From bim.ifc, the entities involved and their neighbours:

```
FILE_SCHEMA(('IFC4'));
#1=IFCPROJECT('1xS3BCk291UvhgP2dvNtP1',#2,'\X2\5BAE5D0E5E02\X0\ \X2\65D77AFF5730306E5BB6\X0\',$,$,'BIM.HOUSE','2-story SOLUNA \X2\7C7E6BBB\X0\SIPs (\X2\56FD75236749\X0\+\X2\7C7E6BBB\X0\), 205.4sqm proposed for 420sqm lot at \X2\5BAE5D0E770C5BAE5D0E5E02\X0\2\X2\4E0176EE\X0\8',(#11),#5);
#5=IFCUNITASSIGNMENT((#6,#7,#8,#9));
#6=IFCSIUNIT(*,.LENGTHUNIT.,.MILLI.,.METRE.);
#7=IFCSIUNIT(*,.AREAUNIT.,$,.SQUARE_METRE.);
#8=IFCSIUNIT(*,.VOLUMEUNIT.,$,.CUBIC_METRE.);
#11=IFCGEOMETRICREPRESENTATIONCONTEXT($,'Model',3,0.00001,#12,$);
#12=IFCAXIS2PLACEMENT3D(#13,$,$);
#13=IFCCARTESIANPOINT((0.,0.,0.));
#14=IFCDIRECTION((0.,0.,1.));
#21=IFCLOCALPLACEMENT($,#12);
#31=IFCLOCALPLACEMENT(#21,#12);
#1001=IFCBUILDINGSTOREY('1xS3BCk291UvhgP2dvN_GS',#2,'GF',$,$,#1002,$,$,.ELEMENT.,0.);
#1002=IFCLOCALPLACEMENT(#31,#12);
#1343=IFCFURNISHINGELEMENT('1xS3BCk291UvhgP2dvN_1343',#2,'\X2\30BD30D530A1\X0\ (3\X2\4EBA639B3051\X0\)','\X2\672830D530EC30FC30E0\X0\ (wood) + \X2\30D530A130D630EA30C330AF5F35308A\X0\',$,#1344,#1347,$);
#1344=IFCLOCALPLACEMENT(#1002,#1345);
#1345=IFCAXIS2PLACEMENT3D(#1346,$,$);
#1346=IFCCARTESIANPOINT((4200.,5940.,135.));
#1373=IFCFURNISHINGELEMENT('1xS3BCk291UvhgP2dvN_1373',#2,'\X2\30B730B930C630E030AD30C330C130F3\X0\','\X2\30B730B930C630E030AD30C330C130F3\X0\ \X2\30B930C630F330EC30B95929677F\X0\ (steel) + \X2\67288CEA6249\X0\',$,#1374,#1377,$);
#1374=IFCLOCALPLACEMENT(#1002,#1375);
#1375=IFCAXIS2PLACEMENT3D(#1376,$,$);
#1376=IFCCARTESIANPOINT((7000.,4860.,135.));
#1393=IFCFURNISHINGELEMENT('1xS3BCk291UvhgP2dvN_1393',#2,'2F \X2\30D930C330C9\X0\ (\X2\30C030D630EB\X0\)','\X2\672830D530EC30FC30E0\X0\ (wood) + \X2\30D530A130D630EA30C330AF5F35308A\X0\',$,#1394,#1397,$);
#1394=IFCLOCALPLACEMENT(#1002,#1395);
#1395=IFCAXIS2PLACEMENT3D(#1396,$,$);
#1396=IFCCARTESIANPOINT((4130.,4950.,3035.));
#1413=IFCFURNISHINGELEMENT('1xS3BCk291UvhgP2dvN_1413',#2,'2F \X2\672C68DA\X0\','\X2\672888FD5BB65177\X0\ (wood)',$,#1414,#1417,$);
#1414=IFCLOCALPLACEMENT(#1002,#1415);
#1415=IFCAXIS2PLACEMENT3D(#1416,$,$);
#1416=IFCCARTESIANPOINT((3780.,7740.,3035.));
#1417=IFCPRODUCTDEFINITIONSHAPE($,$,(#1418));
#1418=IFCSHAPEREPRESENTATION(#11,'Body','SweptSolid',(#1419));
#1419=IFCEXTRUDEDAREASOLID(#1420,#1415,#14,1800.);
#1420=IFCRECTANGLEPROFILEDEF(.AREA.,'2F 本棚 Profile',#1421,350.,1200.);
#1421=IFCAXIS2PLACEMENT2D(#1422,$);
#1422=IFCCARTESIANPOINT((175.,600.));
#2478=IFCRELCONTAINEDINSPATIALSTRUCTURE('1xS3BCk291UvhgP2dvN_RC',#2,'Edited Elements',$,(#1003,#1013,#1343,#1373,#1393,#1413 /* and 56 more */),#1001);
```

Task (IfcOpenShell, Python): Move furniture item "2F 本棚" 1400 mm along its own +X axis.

```python
import ifcopenshell
import ifcopenshell.api.geometry
import ifcopenshell.util.placement

model = ifcopenshell.open("bim.ifc")

item = model.by_guid("1xS3BCk291UvhgP2dvN_1413")
matrix = ifcopenshell.util.placement.get_local_placement(item.ObjectPlacement)
matrix[:3, 3] += matrix[:3, 0] * 1400.0
ifcopenshell.api.geometry.edit_object_placement(model, product=item, matrix=matrix, is_si=False)

print(ifcopenshell.util.placement.get_local_placement(item.ObjectPlacement).round(3) + 0.0)

model.write("bim_edited.ifc")
```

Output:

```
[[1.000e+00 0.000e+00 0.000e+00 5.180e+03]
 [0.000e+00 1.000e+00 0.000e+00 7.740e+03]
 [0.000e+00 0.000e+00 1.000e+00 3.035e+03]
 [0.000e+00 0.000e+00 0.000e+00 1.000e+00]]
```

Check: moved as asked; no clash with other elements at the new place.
